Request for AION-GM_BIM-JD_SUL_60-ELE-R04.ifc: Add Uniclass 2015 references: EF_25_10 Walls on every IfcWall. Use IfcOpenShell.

First a look at what the model holds.

```python
import ifcopenshell

model = ifcopenshell.open("AION-GM_BIM-JD_SUL_60-ELE-R04.ifc")
print(model.schema)
print("classifications:", [c.Name for c in model.by_type("IfcClassification")])
for ifc_class in ("IfcDoor", "IfcRoof", "IfcStair", "IfcWall", "IfcWindow"):
    print(ifc_class, len(model.by_type(ifc_class)))
```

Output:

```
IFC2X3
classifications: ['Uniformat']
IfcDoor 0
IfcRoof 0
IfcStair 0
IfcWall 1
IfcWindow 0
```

```python
import ifcopenshell
import ifcopenshell.api.classification

model = ifcopenshell.open("AION-GM_BIM-JD_SUL_60-ELE-R04.ifc")

# IFC2X3 requires Source and Edition and has no link from the project to the system.
system = model.create_entity("IfcClassification", Source="NBS", Edition="2015", Name="Uniclass 2015")

codes = {
    "IfcWall": ("EF_25_10", "Walls"),
}
for ifc_class, (code, name) in codes.items():
    products = model.by_type(ifc_class)
    ifcopenshell.api.classification.add_reference(
        model, products=products, classification=system, identification=code, name=name
    )
    print(code, len(products))

model.write("AION-GM_BIM-JD_SUL_60-ELE-R04_rev.ifc")
```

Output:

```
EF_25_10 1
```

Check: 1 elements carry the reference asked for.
